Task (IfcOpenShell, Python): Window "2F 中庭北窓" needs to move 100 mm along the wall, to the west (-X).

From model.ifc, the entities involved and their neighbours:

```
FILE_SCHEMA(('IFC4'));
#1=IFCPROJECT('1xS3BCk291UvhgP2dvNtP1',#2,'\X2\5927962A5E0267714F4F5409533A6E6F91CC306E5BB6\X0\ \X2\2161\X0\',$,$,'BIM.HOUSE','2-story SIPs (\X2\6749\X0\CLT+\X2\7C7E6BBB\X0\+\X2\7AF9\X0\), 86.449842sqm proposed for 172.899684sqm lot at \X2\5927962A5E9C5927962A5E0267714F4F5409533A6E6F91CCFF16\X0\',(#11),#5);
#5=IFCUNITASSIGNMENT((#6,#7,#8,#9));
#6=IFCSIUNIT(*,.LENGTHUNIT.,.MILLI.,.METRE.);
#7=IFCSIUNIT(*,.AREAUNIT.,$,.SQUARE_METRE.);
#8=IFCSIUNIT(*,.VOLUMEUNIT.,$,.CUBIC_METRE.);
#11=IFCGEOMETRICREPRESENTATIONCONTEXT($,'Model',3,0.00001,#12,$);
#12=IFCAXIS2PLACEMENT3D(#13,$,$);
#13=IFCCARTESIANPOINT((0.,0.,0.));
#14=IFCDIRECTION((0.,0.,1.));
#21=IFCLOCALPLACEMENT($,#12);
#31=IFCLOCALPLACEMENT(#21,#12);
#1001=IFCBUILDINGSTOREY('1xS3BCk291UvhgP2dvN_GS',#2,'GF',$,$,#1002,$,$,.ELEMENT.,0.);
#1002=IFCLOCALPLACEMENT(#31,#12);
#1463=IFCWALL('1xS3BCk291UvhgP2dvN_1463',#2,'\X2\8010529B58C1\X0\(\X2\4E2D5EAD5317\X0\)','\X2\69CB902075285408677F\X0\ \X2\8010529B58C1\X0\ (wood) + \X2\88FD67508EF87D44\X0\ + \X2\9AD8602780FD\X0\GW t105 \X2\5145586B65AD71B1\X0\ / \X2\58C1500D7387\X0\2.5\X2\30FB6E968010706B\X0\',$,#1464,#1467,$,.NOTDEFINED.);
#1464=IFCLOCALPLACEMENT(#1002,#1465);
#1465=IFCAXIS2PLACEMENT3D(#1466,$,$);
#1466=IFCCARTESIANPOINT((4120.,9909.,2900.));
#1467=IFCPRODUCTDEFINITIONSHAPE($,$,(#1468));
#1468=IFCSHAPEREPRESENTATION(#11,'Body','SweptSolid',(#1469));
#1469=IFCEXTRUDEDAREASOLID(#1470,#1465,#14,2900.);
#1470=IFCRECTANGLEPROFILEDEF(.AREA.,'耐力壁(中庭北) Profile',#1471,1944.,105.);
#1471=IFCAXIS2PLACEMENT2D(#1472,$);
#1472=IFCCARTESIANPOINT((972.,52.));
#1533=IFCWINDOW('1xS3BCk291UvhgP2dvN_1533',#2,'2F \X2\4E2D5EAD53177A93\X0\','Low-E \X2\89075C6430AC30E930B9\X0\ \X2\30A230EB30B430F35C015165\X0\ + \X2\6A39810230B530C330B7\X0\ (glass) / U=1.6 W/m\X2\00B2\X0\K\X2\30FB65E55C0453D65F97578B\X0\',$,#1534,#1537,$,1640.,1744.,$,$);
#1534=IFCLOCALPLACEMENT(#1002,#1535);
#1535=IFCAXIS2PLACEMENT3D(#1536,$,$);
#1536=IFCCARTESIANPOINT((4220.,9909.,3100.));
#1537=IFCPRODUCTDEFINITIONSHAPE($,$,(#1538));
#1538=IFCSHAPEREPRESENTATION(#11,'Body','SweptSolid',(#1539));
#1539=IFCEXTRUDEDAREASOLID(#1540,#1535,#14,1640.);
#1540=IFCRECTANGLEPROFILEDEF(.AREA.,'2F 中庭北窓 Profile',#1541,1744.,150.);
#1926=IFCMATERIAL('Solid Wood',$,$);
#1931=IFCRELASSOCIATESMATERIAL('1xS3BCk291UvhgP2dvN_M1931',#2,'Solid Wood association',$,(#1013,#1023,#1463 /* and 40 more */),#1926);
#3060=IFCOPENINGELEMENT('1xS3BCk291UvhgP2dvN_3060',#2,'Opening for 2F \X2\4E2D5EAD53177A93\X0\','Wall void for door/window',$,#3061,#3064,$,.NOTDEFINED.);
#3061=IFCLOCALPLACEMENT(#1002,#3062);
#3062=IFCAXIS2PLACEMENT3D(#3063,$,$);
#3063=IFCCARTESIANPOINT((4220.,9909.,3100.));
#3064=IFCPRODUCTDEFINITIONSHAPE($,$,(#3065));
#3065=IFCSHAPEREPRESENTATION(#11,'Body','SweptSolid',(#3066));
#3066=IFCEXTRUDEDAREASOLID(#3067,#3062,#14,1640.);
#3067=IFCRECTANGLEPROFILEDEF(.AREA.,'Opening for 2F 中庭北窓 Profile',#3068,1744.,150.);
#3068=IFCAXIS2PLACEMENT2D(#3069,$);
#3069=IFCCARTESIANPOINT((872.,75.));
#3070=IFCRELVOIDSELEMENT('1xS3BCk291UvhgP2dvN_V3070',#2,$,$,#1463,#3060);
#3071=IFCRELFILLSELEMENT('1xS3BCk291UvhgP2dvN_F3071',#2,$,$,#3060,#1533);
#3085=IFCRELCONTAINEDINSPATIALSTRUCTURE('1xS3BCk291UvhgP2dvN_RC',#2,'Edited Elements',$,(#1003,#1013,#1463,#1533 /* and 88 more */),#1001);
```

```python
import ifcopenshell
import ifcopenshell.api.geometry
import ifcopenshell.util.placement
import ifcopenshell.util.unit

model = ifcopenshell.open("model.ifc")
unit_scale = ifcopenshell.util.unit.calculate_unit_scale(model)

window = model.by_id(1533)
opening = window.FillsVoids[0].RelatingOpeningElement
wall = opening.VoidsElements[0].RelatingBuildingElement

wall_matrix = ifcopenshell.util.placement.get_local_placement(wall.ObjectPlacement)
shift = wall_matrix[:3, 0] * -0.1 / unit_scale
before = ifcopenshell.util.placement.get_local_placement(window.ObjectPlacement)[:3, 3].copy()

# The window is not placed relative to its opening, so move both.
for product in (opening, window):
    matrix = ifcopenshell.util.placement.get_local_placement(product.ObjectPlacement)
    matrix[:3, 3] += shift
    ifcopenshell.api.geometry.edit_object_placement(model, product=product, matrix=matrix, is_si=False)

after = ifcopenshell.util.placement.get_local_placement(window.ObjectPlacement)[:3, 3]
print("window moved by", (after - before).round(3) + 0.0)

model.write("model_edited.ifc")
```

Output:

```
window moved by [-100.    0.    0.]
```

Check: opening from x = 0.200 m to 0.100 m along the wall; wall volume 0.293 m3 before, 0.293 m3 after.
